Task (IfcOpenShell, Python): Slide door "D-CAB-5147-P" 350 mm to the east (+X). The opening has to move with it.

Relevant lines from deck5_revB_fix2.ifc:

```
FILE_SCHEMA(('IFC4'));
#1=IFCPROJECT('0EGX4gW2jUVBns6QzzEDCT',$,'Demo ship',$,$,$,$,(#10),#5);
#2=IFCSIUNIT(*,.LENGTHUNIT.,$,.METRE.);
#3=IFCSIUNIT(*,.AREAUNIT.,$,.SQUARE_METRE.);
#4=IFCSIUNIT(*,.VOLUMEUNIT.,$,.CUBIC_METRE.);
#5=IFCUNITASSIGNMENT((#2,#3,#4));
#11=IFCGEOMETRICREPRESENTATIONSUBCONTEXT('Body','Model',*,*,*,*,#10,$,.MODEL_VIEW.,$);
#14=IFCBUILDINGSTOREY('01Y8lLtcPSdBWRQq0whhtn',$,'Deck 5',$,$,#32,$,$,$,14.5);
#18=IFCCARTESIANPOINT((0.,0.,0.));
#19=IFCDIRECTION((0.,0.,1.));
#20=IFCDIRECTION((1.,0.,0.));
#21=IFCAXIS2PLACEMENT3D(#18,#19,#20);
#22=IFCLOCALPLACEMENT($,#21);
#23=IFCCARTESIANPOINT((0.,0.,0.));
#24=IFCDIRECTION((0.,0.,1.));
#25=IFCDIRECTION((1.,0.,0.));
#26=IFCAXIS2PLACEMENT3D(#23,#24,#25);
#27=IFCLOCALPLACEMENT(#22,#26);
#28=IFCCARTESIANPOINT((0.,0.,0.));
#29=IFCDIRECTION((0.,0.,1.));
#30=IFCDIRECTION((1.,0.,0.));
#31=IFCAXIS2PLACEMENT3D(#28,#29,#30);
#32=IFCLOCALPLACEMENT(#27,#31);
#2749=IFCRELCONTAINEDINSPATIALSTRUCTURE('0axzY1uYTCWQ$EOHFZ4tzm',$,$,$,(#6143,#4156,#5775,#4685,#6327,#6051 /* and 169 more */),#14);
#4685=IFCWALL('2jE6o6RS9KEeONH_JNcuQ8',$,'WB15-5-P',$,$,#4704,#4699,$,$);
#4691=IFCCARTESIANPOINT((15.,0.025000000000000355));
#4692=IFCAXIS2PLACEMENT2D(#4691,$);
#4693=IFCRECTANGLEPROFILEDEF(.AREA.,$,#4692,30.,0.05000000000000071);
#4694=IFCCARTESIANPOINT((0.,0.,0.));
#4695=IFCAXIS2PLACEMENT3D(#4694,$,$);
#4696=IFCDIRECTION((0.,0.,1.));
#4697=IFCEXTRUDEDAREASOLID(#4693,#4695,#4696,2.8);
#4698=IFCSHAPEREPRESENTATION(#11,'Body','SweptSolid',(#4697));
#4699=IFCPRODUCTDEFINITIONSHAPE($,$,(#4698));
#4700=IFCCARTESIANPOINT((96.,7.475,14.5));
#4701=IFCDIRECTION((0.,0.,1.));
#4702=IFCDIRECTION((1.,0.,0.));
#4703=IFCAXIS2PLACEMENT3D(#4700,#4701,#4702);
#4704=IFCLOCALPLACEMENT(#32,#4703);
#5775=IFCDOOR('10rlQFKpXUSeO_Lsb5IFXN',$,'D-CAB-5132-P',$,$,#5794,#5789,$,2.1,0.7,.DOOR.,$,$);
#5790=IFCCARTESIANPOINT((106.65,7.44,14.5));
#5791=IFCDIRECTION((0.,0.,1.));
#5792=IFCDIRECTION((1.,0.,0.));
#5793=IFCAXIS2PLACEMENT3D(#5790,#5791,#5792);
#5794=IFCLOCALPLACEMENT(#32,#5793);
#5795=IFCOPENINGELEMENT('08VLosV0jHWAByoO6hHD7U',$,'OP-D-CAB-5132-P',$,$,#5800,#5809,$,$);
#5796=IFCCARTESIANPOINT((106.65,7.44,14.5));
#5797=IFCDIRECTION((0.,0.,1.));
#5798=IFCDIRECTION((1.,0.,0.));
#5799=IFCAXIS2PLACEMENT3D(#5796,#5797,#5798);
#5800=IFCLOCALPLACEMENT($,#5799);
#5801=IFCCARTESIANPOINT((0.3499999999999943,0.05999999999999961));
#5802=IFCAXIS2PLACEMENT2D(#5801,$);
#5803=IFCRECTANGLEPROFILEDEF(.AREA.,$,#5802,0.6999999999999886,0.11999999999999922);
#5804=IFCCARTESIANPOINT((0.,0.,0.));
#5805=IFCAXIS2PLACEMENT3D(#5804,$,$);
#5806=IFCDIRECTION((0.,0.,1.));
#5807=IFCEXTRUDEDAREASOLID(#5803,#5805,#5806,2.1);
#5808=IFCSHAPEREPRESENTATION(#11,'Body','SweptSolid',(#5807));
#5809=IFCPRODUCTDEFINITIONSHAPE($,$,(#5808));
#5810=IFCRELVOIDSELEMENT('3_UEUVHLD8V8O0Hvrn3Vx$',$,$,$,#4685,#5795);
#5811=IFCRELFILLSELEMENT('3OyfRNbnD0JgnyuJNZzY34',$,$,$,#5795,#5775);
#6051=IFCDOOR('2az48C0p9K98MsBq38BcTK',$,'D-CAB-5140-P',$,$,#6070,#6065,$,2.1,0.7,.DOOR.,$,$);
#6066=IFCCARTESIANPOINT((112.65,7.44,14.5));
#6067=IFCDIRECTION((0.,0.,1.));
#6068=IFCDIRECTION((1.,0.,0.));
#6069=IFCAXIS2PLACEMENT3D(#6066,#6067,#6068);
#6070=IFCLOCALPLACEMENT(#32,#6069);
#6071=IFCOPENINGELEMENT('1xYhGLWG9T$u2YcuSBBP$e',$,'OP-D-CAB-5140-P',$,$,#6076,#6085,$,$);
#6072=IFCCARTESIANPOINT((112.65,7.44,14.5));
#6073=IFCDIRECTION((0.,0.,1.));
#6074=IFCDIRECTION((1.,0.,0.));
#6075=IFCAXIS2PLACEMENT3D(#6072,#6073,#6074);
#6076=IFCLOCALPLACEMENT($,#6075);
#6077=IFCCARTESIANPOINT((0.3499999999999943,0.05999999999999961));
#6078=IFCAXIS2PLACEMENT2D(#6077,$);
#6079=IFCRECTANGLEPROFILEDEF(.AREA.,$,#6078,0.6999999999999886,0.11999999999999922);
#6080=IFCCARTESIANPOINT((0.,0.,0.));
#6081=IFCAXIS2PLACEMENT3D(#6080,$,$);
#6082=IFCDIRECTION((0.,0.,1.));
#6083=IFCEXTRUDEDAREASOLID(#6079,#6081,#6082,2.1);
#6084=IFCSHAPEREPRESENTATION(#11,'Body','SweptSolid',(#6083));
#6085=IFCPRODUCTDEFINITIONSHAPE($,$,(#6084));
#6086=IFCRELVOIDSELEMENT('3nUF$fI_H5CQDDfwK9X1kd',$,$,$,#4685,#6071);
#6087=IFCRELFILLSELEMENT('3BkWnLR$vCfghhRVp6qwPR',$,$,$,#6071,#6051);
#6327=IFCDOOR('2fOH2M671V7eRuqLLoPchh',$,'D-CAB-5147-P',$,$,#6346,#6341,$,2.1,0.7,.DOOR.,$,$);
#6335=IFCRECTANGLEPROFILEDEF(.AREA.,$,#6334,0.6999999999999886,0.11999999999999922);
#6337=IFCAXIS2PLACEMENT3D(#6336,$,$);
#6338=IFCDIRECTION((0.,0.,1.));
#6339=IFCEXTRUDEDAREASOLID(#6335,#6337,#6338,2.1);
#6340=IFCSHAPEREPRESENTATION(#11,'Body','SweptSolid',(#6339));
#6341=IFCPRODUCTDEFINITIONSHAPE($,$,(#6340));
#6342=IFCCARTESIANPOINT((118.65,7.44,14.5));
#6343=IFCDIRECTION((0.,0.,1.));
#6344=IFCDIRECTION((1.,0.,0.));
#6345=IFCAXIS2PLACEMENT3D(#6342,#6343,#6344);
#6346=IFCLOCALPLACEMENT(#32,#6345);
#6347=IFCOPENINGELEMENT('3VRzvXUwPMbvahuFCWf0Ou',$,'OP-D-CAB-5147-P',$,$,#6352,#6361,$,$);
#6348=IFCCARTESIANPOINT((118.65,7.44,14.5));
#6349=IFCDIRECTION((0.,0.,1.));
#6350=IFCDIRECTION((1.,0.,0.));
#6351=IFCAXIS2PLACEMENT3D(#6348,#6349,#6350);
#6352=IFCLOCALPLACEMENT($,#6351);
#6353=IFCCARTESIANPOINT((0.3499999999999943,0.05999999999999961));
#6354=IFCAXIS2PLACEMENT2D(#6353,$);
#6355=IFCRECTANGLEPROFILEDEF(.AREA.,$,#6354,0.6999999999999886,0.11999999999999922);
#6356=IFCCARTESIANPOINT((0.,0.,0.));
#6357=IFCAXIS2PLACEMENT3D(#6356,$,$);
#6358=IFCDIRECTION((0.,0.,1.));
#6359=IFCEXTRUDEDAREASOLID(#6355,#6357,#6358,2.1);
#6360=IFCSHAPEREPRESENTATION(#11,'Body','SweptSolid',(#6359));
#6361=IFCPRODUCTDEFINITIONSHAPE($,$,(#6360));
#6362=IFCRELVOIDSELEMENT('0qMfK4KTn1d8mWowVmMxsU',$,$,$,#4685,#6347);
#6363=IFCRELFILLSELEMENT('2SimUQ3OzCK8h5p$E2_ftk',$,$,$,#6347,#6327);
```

```python
import ifcopenshell
import ifcopenshell.api.geometry
import ifcopenshell.util.placement
import ifcopenshell.util.unit

model = ifcopenshell.open("deck5_revB_fix2.ifc")
unit_scale = ifcopenshell.util.unit.calculate_unit_scale(model)

door = model.by_guid("2fOH2M671V7eRuqLLoPchh")
opening = door.FillsVoids[0].RelatingOpeningElement
wall = opening.VoidsElements[0].RelatingBuildingElement

wall_matrix = ifcopenshell.util.placement.get_local_placement(wall.ObjectPlacement)
shift = wall_matrix[:3, 0] * 0.35 / unit_scale
before = ifcopenshell.util.placement.get_local_placement(door.ObjectPlacement)[:3, 3].copy()

# The door is not placed relative to its opening, so move both.
for product in (opening, door):
    matrix = ifcopenshell.util.placement.get_local_placement(product.ObjectPlacement)
    matrix[:3, 3] += shift
    ifcopenshell.api.geometry.edit_object_placement(model, product=product, matrix=matrix, is_si=False)

after = ifcopenshell.util.placement.get_local_placement(door.ObjectPlacement)[:3, 3]
print("door moved by", (after - before).round(3) + 0.0)

model.write("deck5_revB_fix2_edited.ifc")
```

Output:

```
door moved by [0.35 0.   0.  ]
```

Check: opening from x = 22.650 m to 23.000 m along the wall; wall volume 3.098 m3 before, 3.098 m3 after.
